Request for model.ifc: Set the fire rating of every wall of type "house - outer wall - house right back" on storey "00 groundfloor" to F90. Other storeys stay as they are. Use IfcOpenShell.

First a look at what the model holds.

```python
import ifcopenshell
import ifcopenshell.util.element

model = ifcopenshell.open("model.ifc")
print(model.schema)
storey = next(s for s in model.by_type("IfcBuildingStorey") if s.Name == "00 groundfloor")
walls = [e for e in ifcopenshell.util.element.get_decomposition(storey) if e.is_a("IfcWall")]
seen = {}
for e in walls:
    element_type = ifcopenshell.util.element.get_type(e)
    key = (element_type.Name if element_type != e and element_type else None, ifcopenshell.util.element.get_pset(e, "Pset_WallCommon", "FireRating"))
    seen[key] = seen.get(key, 0) + 1
for (name, value), count in sorted(seen.items(), key=str):
    print(count, "x", name, "|", value)
```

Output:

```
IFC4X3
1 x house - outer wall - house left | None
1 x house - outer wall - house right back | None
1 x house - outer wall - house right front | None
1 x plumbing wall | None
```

```python
import ifcopenshell
import ifcopenshell.api.pset
import ifcopenshell.util.element

model = ifcopenshell.open("model.ifc")

storey = next(s for s in model.by_type("IfcBuildingStorey") if s.Name == "00 groundfloor")
walls = [e for e in ifcopenshell.util.element.get_decomposition(storey) if e.is_a("IfcWall")]

count = 0
for e in walls:
    element_type = ifcopenshell.util.element.get_type(e)
    if element_type in (None, e) or element_type.Name != "house - outer wall - house right back":
        continue
    # add_pset returns the element's existing set when there is one.
    pset = ifcopenshell.api.pset.add_pset(model, product=e, name="Pset_WallCommon")
    ifcopenshell.api.pset.edit_pset(model, pset=pset, properties={"FireRating": "F90"})
    count += 1

print(count, "walls updated")

model.write("model_v2.ifc")
```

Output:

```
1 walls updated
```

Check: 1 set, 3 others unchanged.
